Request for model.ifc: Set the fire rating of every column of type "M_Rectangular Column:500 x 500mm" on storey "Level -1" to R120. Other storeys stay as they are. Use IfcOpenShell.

First a look at what the model holds.

```python
import ifcopenshell
import ifcopenshell.util.element

model = ifcopenshell.open("model.ifc")
print(model.schema)
storey = next(s for s in model.by_type("IfcBuildingStorey") if s.Name == "Level -1")
columns = [e for e in ifcopenshell.util.element.get_decomposition(storey) if e.is_a("IfcColumn")]
seen = {}
for e in columns:
    element_type = ifcopenshell.util.element.get_type(e)
    key = (element_type.Name if element_type != e and element_type else None, ifcopenshell.util.element.get_pset(e, "Pset_ColumnCommon", "FireRating"))
    seen[key] = seen.get(key, 0) + 1
for (name, value), count in sorted(seen.items(), key=str):
    print(count, "x", name, "|", value)
```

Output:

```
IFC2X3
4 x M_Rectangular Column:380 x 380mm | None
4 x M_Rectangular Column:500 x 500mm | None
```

```python
import ifcopenshell
import ifcopenshell.api.pset
import ifcopenshell.util.element

model = ifcopenshell.open("model.ifc")

storey = next(s for s in model.by_type("IfcBuildingStorey") if s.Name == "Level -1")
columns = [e for e in ifcopenshell.util.element.get_decomposition(storey) if e.is_a("IfcColumn")]

count = 0
for e in columns:
    element_type = ifcopenshell.util.element.get_type(e)
    if element_type in (None, e) or element_type.Name != "M_Rectangular Column:500 x 500mm":
        continue
    # add_pset returns the element's existing set when there is one.
    pset = ifcopenshell.api.pset.add_pset(model, product=e, name="Pset_ColumnCommon")
    ifcopenshell.api.pset.edit_pset(model, pset=pset, properties={"FireRating": "R120"})
    count += 1

print(count, "columns updated")

model.write("model-out.ifc")
```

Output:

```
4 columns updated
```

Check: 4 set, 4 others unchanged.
